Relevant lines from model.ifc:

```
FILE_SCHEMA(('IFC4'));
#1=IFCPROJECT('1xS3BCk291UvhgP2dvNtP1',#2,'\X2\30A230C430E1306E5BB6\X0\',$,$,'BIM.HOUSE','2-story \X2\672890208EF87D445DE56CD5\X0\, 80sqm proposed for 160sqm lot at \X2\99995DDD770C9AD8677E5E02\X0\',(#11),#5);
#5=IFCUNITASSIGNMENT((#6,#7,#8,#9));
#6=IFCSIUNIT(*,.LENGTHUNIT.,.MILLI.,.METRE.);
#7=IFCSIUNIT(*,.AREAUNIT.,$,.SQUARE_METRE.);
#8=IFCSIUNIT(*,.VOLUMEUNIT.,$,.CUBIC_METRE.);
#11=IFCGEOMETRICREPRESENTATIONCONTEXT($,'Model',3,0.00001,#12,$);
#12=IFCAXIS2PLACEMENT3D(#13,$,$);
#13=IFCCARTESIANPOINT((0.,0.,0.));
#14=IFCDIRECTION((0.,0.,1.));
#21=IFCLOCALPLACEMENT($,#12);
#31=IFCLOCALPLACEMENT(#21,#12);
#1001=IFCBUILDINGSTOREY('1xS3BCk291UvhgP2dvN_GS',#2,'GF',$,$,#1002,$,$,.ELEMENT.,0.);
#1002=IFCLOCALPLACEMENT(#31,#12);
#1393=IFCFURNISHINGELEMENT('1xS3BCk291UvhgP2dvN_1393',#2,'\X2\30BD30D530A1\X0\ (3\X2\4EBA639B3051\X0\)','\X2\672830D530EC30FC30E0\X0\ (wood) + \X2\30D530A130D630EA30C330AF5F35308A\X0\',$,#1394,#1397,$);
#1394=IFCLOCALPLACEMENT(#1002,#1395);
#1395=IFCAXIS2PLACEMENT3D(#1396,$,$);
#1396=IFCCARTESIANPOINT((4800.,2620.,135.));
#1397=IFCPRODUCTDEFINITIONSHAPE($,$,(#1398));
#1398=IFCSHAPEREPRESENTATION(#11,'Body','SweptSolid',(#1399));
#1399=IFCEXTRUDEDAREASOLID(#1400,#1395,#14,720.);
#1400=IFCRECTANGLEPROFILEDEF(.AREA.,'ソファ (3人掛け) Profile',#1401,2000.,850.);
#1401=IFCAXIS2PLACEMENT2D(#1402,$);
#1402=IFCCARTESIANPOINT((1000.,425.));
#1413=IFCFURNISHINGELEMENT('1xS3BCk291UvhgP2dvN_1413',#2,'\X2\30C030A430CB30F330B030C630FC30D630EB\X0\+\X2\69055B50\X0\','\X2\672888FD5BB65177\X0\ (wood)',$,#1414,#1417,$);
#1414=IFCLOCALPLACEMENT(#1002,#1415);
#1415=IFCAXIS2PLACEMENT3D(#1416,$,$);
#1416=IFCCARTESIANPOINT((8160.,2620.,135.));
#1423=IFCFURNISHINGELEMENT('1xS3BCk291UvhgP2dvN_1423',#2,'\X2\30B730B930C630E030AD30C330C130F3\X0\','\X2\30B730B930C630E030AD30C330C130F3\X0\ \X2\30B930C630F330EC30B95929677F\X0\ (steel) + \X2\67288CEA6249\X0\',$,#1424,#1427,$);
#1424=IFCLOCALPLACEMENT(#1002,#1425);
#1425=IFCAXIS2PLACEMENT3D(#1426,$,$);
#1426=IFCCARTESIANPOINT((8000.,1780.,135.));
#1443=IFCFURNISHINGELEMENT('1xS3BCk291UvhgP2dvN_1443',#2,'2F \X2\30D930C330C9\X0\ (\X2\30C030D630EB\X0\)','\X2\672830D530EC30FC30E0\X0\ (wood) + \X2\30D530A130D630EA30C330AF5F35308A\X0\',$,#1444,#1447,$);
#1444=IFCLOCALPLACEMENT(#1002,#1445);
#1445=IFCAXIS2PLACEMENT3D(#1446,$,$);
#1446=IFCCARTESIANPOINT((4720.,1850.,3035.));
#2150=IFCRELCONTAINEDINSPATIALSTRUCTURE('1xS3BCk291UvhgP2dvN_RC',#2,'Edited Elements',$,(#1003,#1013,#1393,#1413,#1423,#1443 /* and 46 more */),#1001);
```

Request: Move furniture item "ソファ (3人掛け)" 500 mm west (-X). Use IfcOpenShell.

```python
import ifcopenshell
import ifcopenshell.api.geometry
import ifcopenshell.util.placement
import ifcopenshell.util.unit

model = ifcopenshell.open("model.ifc")
unit_scale = ifcopenshell.util.unit.calculate_unit_scale(model)

item = model.by_guid("1xS3BCk291UvhgP2dvN_1393")
matrix = ifcopenshell.util.placement.get_local_placement(item.ObjectPlacement)
matrix[0, 3] -= 0.5 / unit_scale
ifcopenshell.api.geometry.edit_object_placement(model, product=item, matrix=matrix, is_si=False)

print(ifcopenshell.util.placement.get_local_placement(item.ObjectPlacement).round(3) + 0.0)

model.write("model_rev.ifc")
```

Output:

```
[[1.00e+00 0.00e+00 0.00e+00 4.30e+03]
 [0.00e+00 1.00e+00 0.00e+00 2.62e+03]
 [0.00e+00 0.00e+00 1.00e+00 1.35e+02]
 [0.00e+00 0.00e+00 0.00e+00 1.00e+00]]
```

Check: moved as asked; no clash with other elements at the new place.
